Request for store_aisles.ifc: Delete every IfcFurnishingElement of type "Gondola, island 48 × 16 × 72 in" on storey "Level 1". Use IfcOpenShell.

First a look at what the model holds.

```python
import ifcopenshell
import ifcopenshell.util.element

model = ifcopenshell.open("store_aisles.ifc")
print(model.schema)
storey = next(s for s in model.by_type("IfcBuildingStorey") if s.Name == "Level 1")
furniture = [e for e in ifcopenshell.util.element.get_decomposition(storey) if e.is_a("IfcFurnishingElement")]
seen = {}
for e in furniture:
    element_type = ifcopenshell.util.element.get_type(e)
    name = element_type.Name if element_type not in (None, e) else None
    seen[name] = seen.get(name, 0) + 1
for name, count in sorted(seen.items(), key=str):
    print(count, "x", name)
```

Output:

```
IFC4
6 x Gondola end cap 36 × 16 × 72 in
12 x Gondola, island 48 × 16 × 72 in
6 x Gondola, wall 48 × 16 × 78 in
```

```python
import ifcopenshell
import ifcopenshell.api.root
import ifcopenshell.util.element

model = ifcopenshell.open("store_aisles.ifc")

storey = next(s for s in model.by_type("IfcBuildingStorey") if s.Name == "Level 1")
furniture = [e for e in ifcopenshell.util.element.get_decomposition(storey) if e.is_a("IfcFurnishingElement")]
targets = [e for e in furniture if (t := ifcopenshell.util.element.get_type(e)) not in (None, e) and t.Name == "Gondola, island 48 × 16 × 72 in"]

for e in targets:
    ifcopenshell.api.root.remove_product(model, product=e)
print(len(targets), "removed")

model.write("store_aisles_updated.ifc")
```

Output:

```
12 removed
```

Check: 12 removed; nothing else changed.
